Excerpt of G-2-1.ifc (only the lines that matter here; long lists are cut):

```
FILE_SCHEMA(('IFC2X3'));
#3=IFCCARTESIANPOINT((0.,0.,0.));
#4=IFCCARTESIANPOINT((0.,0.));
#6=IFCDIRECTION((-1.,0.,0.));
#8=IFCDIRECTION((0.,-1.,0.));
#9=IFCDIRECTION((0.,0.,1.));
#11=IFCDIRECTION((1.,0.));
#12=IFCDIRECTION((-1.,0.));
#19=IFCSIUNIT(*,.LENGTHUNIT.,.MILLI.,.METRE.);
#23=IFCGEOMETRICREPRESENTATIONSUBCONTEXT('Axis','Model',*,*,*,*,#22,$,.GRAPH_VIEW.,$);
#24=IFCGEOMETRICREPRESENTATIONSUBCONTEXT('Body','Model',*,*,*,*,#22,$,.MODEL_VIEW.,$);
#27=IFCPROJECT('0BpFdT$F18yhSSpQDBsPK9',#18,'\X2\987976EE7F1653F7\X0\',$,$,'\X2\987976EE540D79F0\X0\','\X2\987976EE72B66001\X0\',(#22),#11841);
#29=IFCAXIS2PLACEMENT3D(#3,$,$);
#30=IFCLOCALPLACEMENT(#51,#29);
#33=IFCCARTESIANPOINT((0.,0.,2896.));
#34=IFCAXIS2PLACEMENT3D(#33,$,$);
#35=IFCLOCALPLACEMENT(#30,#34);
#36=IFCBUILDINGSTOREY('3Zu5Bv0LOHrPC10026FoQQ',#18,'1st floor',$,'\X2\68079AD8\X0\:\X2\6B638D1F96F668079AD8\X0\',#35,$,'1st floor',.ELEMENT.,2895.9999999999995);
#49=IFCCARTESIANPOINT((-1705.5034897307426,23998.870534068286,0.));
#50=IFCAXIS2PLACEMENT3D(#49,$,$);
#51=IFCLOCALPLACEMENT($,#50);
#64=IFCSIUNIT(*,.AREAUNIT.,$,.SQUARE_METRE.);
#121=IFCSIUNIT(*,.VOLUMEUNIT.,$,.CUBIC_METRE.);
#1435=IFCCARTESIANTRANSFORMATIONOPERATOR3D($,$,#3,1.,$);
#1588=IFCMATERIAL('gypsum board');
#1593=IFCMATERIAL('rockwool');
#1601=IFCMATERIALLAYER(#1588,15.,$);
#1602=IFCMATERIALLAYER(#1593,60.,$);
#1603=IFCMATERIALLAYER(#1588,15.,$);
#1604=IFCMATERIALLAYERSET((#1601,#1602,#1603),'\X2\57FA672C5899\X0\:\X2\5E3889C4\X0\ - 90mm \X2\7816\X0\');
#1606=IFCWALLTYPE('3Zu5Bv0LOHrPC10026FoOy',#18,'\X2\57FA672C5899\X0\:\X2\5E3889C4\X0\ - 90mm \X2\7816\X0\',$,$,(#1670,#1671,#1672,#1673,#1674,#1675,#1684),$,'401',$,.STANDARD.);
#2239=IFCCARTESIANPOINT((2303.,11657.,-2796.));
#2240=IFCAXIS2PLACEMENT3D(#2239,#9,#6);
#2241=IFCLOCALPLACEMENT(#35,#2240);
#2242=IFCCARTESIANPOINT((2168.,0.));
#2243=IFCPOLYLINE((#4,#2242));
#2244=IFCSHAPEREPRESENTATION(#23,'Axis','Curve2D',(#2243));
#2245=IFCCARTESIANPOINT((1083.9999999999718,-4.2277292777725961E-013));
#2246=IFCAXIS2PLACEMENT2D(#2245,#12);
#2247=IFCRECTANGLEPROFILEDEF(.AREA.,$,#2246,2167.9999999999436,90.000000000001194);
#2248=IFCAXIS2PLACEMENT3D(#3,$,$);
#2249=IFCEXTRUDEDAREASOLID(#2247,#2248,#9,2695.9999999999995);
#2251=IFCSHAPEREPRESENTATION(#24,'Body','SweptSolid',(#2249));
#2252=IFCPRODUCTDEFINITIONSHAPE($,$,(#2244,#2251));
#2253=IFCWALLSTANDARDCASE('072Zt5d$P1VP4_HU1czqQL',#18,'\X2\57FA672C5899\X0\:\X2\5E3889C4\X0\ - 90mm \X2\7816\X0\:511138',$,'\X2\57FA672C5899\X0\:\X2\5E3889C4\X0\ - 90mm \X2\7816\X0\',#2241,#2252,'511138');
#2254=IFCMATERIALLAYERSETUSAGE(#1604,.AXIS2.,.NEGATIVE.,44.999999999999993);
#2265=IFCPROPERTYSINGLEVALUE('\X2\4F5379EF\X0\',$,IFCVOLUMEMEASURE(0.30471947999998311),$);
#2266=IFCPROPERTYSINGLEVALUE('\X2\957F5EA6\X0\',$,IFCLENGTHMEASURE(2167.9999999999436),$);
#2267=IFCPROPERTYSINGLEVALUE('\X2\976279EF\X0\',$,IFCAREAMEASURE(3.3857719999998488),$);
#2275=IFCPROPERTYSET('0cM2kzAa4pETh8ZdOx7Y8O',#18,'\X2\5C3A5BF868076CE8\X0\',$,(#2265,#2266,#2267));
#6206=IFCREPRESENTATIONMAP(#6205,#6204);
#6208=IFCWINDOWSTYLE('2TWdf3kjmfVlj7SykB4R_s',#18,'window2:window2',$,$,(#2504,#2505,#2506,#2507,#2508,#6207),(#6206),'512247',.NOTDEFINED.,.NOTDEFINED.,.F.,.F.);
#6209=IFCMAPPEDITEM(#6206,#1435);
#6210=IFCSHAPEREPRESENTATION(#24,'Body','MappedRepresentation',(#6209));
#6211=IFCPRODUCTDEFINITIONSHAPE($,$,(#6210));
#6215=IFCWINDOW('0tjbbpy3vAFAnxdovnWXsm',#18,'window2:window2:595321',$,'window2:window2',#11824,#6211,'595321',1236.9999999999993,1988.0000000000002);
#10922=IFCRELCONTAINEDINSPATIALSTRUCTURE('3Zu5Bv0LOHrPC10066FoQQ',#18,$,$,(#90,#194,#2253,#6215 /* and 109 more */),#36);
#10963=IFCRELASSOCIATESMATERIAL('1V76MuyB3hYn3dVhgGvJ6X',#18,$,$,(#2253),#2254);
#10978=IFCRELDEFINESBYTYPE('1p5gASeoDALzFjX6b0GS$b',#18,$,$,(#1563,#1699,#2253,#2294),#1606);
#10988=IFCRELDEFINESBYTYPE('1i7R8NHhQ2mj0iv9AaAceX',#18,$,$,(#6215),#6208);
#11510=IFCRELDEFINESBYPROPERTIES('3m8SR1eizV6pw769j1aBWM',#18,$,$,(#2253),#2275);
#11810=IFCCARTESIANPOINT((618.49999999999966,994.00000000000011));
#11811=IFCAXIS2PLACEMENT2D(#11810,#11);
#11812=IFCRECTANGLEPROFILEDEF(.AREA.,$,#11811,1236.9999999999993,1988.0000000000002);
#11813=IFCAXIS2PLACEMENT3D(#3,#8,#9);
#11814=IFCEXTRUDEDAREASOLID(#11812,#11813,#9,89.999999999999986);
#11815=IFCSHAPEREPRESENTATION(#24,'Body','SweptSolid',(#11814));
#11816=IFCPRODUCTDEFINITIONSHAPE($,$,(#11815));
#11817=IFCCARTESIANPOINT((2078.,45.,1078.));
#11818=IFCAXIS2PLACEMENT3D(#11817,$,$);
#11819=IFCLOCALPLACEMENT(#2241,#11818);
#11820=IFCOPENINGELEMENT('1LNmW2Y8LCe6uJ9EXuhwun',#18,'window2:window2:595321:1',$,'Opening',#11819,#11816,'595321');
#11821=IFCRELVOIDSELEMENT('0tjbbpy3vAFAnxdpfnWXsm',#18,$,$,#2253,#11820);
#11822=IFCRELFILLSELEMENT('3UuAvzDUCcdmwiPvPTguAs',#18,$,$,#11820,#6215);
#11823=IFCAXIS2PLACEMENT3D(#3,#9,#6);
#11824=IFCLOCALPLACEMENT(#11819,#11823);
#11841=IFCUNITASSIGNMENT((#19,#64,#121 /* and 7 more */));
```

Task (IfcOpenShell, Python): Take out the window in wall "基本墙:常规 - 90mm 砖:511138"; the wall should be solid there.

```python
import ifcopenshell
import ifcopenshell.api.feature
import ifcopenshell.api.pset
import ifcopenshell.api.root
import ifcopenshell.geom
import ifcopenshell.util.element
import ifcopenshell.util.shape
import ifcopenshell.util.unit

model = ifcopenshell.open("G-2-1.ifc")
area_scale = ifcopenshell.util.unit.calculate_unit_scale(model, "AREAUNIT")
volume_scale = ifcopenshell.util.unit.calculate_unit_scale(model, "VOLUMEUNIT")
settings = ifcopenshell.geom.settings()


def volume(element):
    """Net volume in cubic metres, openings subtracted."""
    shape = ifcopenshell.geom.create_shape(settings, element)
    return ifcopenshell.util.shape.get_volume(shape.geometry)


window = model.by_guid("0tjbbpy3vAFAnxdovnWXsm")
opening = window.FillsVoids[0].RelatingOpeningElement
wall = opening.VoidsElements[0].RelatingBuildingElement
before = volume(wall)

ifcopenshell.api.root.remove_product(model, product=window)
ifcopenshell.api.feature.remove_feature(model, feature=opening)

after = volume(wall)
thickness = 0.09  # wall thickness in metres

# Update the wall's stored quantities.
pset = model.by_id(ifcopenshell.util.element.get_pset(wall, "尺寸标注", should_inherit=False)["id"])
ifcopenshell.api.pset.edit_pset(model, pset=pset, properties={
    "体积": model.create_entity("IfcVolumeMeasure", after / volume_scale),
    "面积": model.create_entity("IfcAreaMeasure", after / thickness / area_scale),
})

print(f"wall volume {before:.3f} -> {after:.3f} m3")

model.write("G-2-1_updated.ifc")
```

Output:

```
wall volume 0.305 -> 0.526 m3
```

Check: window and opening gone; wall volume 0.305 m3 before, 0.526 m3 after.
